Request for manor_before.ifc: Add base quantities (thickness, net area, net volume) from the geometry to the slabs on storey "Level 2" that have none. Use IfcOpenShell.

First a look at what the model holds.

```python
import ifcopenshell
import ifcopenshell.util.element
import ifcopenshell.util.unit

model = ifcopenshell.open("manor_before.ifc")
print(model.schema)
for unit_type in ("LENGTHUNIT", "AREAUNIT", "VOLUMEUNIT"):
    print(unit_type, ifcopenshell.util.unit.calculate_unit_scale(model, unit_type))
storey = next(s for s in model.by_type("IfcBuildingStorey") if s.Name == "Level 2")
slabs = [e for e in ifcopenshell.util.element.get_decomposition(storey) if e.is_a("IfcSlab")]
for e in sorted(slabs, key=lambda e: e.id()):
    print(e.id(), e.is_a(), e.Name, list(ifcopenshell.util.element.get_psets(e, qtos_only=True)), sep=" | ")
```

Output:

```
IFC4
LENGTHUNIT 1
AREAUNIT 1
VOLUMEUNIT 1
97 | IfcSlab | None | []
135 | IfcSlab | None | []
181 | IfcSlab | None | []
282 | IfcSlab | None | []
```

```python
import ifcopenshell
import ifcopenshell.api.pset
import ifcopenshell.geom
import ifcopenshell.util.element
import ifcopenshell.util.shape
import ifcopenshell.util.unit

model = ifcopenshell.open("manor_before.ifc")
unit_scale = ifcopenshell.util.unit.calculate_unit_scale(model)
area_scale = ifcopenshell.util.unit.calculate_unit_scale(model, "AREAUNIT")
volume_scale = ifcopenshell.util.unit.calculate_unit_scale(model, "VOLUMEUNIT")
settings = ifcopenshell.geom.settings()

storey = next(s for s in model.by_type("IfcBuildingStorey") if s.Name == "Level 2")
slabs = [e for e in ifcopenshell.util.element.get_decomposition(storey) if e.is_a("IfcSlab")]

for e in sorted(slabs, key=lambda e: e.id()):
    if ifcopenshell.util.element.get_psets(e, qtos_only=True, should_inherit=False):
        continue
    # Geometry comes back in metres, in the element's own axes.
    shape = ifcopenshell.geom.create_shape(settings, e)
    values = {
        "Width": ifcopenshell.util.shape.get_z(shape.geometry) / unit_scale,
        "NetArea": ifcopenshell.util.shape.get_footprint_area(shape.geometry) / area_scale,
        "NetVolume": ifcopenshell.util.shape.get_volume(shape.geometry) / volume_scale,
    }
    qto = ifcopenshell.api.pset.add_qto(model, product=e, name="Qto_SlabBaseQuantities")
    ifcopenshell.api.pset.edit_qto(model, qto=qto, properties=values)
    print(e.id(), {k: round(v, 3) for k, v in values.items()})

model.write("manor_before-out.ifc")
```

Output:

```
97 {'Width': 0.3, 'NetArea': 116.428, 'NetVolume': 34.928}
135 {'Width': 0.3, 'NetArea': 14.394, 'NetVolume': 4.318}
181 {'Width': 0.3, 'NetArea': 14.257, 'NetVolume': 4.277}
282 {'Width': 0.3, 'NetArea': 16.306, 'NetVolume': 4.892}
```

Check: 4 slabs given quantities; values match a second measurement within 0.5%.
